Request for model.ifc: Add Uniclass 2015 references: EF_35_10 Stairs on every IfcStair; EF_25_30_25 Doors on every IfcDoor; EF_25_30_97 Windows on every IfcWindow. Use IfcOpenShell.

First a look at what the model holds.

```python
import ifcopenshell

model = ifcopenshell.open("model.ifc")
print(model.schema)
print("classifications:", [c.Name for c in model.by_type("IfcClassification")])
for ifc_class in ("IfcDoor", "IfcRoof", "IfcStair", "IfcWall", "IfcWindow"):
    print(ifc_class, len(model.by_type(ifc_class)))
```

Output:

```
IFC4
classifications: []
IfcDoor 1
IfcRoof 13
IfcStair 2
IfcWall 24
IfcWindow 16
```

```python
import ifcopenshell
import ifcopenshell.api.classification

model = ifcopenshell.open("model.ifc")

system = ifcopenshell.api.classification.add_classification(model, classification="Uniclass 2015")

codes = {
    "IfcStair": ("EF_35_10", "Stairs"),
    "IfcDoor": ("EF_25_30_25", "Doors"),
    "IfcWindow": ("EF_25_30_97", "Windows"),
}
for ifc_class, (code, name) in codes.items():
    products = model.by_type(ifc_class)
    ifcopenshell.api.classification.add_reference(
        model, products=products, classification=system, identification=code, name=name
    )
    print(code, len(products))

model.write("model_edited.ifc")
```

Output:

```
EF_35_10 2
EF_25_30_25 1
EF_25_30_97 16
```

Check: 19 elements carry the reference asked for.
